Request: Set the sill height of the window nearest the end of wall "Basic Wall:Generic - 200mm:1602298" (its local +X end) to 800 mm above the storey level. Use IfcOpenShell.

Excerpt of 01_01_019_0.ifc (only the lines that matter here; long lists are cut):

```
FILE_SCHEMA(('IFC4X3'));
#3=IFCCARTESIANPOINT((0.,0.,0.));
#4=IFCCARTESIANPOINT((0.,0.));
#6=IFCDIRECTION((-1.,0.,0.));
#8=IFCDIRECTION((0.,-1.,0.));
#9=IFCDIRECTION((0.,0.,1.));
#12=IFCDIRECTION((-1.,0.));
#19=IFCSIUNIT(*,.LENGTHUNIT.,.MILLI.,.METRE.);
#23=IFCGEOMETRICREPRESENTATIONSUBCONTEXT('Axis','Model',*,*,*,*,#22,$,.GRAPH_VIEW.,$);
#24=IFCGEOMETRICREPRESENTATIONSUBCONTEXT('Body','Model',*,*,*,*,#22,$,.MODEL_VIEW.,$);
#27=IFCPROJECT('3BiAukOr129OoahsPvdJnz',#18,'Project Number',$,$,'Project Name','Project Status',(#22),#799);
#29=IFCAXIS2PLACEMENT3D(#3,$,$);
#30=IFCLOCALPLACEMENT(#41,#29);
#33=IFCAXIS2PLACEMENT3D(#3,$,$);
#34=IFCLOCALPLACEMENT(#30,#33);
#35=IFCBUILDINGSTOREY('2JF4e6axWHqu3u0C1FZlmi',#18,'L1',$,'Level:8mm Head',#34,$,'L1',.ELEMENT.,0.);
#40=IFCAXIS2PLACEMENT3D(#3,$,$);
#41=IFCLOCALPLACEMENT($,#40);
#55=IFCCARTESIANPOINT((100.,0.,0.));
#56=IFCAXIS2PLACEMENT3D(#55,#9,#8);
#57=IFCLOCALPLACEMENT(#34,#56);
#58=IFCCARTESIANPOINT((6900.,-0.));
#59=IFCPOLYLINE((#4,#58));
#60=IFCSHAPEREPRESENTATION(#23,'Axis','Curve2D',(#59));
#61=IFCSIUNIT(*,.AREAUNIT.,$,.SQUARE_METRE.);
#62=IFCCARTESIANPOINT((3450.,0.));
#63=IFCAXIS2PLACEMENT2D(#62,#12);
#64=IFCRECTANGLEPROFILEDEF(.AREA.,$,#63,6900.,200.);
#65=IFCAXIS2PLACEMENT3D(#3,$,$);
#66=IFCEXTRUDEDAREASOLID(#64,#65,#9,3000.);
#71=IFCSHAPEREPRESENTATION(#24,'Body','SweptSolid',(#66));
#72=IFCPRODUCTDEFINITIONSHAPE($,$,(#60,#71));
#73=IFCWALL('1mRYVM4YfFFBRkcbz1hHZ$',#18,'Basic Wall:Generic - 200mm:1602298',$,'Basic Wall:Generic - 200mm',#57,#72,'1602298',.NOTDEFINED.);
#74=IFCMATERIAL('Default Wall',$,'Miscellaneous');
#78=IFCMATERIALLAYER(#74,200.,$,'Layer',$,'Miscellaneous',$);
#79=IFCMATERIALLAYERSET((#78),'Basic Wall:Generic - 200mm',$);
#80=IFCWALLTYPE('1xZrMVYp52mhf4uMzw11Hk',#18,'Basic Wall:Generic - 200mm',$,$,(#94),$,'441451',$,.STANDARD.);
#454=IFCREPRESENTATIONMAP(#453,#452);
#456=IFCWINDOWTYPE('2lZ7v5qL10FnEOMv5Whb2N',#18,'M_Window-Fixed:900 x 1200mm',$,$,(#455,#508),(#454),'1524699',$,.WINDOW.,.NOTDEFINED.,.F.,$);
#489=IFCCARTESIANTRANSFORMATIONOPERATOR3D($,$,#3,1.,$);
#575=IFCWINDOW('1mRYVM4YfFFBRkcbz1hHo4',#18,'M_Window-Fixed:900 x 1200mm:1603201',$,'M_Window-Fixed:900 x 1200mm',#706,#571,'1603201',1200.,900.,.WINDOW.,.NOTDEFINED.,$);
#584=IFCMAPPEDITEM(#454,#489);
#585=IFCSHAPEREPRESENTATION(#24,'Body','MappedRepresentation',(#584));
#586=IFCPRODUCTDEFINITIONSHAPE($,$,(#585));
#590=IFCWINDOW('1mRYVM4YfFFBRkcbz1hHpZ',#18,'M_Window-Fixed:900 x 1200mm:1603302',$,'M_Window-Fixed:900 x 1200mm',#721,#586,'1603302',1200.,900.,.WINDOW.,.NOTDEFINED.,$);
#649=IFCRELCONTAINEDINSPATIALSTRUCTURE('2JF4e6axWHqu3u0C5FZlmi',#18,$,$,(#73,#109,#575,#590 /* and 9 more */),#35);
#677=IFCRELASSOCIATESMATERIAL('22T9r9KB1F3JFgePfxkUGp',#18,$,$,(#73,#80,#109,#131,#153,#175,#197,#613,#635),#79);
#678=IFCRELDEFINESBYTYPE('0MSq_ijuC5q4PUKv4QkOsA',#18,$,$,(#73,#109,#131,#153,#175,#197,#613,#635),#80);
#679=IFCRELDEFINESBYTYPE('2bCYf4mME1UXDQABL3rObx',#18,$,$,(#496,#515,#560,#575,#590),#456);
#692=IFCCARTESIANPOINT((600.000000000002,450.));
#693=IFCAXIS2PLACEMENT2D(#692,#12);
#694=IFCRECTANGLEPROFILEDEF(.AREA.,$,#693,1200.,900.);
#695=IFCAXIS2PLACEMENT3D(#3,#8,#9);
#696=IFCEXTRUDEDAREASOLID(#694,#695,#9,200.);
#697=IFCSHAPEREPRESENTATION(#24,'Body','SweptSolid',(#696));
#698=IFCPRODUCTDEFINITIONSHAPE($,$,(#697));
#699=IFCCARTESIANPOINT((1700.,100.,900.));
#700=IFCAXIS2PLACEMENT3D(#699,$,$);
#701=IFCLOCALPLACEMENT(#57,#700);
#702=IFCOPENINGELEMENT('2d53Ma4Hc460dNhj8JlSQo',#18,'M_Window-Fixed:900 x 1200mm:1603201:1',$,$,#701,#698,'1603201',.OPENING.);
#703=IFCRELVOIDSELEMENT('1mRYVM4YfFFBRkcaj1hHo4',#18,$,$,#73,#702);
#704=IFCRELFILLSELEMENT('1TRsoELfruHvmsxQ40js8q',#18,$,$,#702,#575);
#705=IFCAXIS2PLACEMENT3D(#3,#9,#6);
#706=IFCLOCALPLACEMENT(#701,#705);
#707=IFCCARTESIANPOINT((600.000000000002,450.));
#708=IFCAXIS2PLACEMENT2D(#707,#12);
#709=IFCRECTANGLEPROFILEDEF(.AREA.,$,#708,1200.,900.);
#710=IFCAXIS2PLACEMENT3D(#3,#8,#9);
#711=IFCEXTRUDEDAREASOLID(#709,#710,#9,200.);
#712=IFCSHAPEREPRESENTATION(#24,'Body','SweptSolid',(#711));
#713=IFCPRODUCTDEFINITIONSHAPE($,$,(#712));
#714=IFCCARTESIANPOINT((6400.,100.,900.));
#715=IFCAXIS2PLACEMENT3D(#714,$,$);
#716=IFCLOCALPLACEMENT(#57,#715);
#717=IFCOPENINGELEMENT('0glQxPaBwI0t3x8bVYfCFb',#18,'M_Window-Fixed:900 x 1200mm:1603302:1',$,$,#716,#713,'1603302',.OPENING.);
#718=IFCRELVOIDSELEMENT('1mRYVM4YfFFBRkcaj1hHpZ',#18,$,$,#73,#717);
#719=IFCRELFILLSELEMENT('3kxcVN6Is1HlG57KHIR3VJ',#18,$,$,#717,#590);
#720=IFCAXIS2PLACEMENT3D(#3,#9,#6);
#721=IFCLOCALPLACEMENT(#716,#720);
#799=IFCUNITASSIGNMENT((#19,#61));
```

```python
import numpy as np
import ifcopenshell
import ifcopenshell.api.geometry
import ifcopenshell.geom
import ifcopenshell.util.element
import ifcopenshell.util.placement
import ifcopenshell.util.shape
import ifcopenshell.util.unit

model = ifcopenshell.open("01_01_019_0.ifc")
unit_scale = ifcopenshell.util.unit.calculate_unit_scale(model)

window = model.by_guid("1mRYVM4YfFFBRkcbz1hHpZ")
opening = window.FillsVoids[0].RelatingOpeningElement
storey = ifcopenshell.util.element.get_container(window, ifc_class="IfcBuildingStorey")
level = ifcopenshell.util.placement.get_local_placement(storey.ObjectPlacement)[2, 3]

# The opening's origin need not be at the sill, so measure its lowest point.
shape = ifcopenshell.geom.create_shape(ifcopenshell.geom.settings(), opening)
bottom = ifcopenshell.util.shape.get_shape_bottom_elevation(shape, shape.geometry) / unit_scale
dz = level + 800.0 - bottom

shift = np.array([0.0, 0.0, dz])
# The window is placed relative to its opening, so it follows when the opening moves.
matrix = ifcopenshell.util.placement.get_local_placement(opening.ObjectPlacement)
matrix[:3, 3] += shift
ifcopenshell.api.geometry.edit_object_placement(
    model, product=opening, matrix=matrix, is_si=False, should_transform_children=True
)

print(f"moved by {dz * unit_scale:+.3f} m")

model.write("01_01_019_0_v2.ifc")
```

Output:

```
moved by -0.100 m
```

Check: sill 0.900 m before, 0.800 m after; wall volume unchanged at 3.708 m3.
